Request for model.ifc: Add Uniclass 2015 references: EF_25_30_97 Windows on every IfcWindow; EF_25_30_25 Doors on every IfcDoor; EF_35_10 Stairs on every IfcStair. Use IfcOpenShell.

First a look at what the model holds.

```python
import ifcopenshell

model = ifcopenshell.open("model.ifc")
print(model.schema)
print("classifications:", [c.Name for c in model.by_type("IfcClassification")])
for ifc_class in ("IfcDoor", "IfcRoof", "IfcStair", "IfcWall", "IfcWindow"):
    print(ifc_class, len(model.by_type(ifc_class)))
```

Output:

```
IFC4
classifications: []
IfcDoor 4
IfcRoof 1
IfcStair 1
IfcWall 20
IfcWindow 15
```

```python
import ifcopenshell
import ifcopenshell.api.classification

model = ifcopenshell.open("model.ifc")

system = ifcopenshell.api.classification.add_classification(model, classification="Uniclass 2015")

codes = {
    "IfcWindow": ("EF_25_30_97", "Windows"),
    "IfcDoor": ("EF_25_30_25", "Doors"),
    "IfcStair": ("EF_35_10", "Stairs"),
}
for ifc_class, (code, name) in codes.items():
    products = model.by_type(ifc_class)
    ifcopenshell.api.classification.add_reference(
        model, products=products, classification=system, identification=code, name=name
    )
    print(code, len(products))

model.write("model_v2.ifc")
```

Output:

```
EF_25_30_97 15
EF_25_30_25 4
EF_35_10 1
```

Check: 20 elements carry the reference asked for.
